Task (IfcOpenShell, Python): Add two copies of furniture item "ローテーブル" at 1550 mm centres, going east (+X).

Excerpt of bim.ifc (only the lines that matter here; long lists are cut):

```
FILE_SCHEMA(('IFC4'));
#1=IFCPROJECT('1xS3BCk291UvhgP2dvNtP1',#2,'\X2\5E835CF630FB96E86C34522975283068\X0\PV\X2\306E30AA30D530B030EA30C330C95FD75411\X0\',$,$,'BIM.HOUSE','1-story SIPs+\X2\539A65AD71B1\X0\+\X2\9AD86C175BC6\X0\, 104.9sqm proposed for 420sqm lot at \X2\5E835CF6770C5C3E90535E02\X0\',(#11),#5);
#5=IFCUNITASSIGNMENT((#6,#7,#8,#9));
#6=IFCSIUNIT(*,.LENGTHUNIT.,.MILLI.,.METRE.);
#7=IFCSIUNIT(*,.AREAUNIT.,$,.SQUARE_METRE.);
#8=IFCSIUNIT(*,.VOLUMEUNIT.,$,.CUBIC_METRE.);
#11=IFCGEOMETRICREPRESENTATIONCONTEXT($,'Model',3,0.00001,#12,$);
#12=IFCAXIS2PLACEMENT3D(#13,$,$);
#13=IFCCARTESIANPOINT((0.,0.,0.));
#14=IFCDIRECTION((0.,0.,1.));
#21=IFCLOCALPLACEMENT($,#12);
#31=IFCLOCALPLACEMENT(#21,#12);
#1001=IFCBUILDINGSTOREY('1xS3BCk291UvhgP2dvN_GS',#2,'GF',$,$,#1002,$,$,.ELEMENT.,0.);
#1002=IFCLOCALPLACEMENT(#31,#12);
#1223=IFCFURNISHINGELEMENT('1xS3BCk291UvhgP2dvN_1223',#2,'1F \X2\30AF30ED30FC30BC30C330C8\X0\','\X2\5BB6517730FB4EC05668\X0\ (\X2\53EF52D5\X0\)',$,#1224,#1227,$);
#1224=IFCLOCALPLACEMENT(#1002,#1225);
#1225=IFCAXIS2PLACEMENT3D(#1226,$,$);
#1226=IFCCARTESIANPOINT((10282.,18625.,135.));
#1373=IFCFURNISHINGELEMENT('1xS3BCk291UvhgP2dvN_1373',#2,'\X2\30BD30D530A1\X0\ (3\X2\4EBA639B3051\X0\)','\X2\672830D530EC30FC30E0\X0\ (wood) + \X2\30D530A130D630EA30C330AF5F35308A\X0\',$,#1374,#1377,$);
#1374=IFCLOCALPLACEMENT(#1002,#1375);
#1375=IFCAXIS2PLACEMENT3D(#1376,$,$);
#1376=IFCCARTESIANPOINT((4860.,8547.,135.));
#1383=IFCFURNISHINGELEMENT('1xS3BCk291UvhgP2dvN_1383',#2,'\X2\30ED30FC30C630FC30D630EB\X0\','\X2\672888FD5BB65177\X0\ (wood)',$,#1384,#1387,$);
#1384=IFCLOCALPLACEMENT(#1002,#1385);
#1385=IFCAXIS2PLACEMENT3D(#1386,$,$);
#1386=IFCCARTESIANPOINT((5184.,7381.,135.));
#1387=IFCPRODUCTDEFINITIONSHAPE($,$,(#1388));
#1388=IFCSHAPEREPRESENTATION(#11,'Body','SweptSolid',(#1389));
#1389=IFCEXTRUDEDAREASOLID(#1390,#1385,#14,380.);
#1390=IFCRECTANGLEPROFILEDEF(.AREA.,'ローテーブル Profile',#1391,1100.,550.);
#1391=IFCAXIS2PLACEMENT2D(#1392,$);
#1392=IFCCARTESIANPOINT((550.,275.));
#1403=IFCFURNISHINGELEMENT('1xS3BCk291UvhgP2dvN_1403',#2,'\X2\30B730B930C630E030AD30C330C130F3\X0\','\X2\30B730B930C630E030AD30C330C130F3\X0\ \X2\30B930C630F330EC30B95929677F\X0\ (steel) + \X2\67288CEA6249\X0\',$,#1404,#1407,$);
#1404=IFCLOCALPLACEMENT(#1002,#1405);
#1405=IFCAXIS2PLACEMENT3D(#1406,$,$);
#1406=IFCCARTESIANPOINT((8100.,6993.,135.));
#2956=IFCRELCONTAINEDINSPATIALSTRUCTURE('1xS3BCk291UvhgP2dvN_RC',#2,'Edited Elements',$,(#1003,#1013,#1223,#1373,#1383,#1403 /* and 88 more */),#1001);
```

```python
import numpy as np
import ifcopenshell
import ifcopenshell.api.geometry
import ifcopenshell.api.root
import ifcopenshell.util.element
import ifcopenshell.util.placement

model = ifcopenshell.open("bim.ifc")


def reuse_history(source, copy):
    """copy_class also copies each property set's owner history, people and application; keep the originals."""
    for rel in copy.IsDefinedBy:
        if rel.is_a("IfcRelDefinesByProperties") and (history := rel.RelatingPropertyDefinition.OwnerHistory):
            rel.RelatingPropertyDefinition.OwnerHistory = source.OwnerHistory
            ifcopenshell.util.element.remove_deep2(model, history)


source = model.by_guid("1xS3BCk291UvhgP2dvN_1383")
base = ifcopenshell.util.placement.get_local_placement(source.ObjectPlacement)
step = np.array([1.0, 0.0, 0.0]) * 1550.0

for i in range(1, 3):
    copy = ifcopenshell.api.root.copy_class(model, product=source)
    copy.Representation = ifcopenshell.util.element.copy_deep(
        model, source.Representation, exclude=["IfcGeometricRepresentationContext", "IfcRepresentationMap"]
    )
    reuse_history(source, copy)
    matrix = base.copy()
    matrix[:3, 3] += i * step
    print("added at", matrix[:3, 3].round(3) + 0.0)
    ifcopenshell.api.geometry.edit_object_placement(model, product=copy, matrix=matrix, is_si=False)

model.write("bim_updated.ifc")
```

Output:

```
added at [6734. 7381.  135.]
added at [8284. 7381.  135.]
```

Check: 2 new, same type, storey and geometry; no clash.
